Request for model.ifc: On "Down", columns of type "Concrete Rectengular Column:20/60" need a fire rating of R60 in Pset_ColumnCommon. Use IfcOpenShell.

First a look at what the model holds.

```python
import ifcopenshell
import ifcopenshell.util.element

model = ifcopenshell.open("model.ifc")
print(model.schema)
storey = next(s for s in model.by_type("IfcBuildingStorey") if s.Name == "Down")
columns = [e for e in ifcopenshell.util.element.get_decomposition(storey) if e.is_a("IfcColumn")]
seen = {}
for e in columns:
    element_type = ifcopenshell.util.element.get_type(e)
    key = (element_type.Name if element_type != e and element_type else None, ifcopenshell.util.element.get_pset(e, "Pset_ColumnCommon", "FireRating"))
    seen[key] = seen.get(key, 0) + 1
for (name, value), count in sorted(seen.items(), key=str):
    print(count, "x", name, "|", value)
```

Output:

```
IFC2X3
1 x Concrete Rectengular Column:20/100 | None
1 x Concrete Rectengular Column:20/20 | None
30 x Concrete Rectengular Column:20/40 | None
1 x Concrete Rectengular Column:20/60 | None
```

```python
import ifcopenshell
import ifcopenshell.api.pset
import ifcopenshell.util.element

model = ifcopenshell.open("model.ifc")

storey = next(s for s in model.by_type("IfcBuildingStorey") if s.Name == "Down")
columns = [e for e in ifcopenshell.util.element.get_decomposition(storey) if e.is_a("IfcColumn")]

count = 0
for e in columns:
    element_type = ifcopenshell.util.element.get_type(e)
    if element_type in (None, e) or element_type.Name != "Concrete Rectengular Column:20/60":
        continue
    # add_pset returns the element's existing set when there is one.
    pset = ifcopenshell.api.pset.add_pset(model, product=e, name="Pset_ColumnCommon")
    ifcopenshell.api.pset.edit_pset(model, pset=pset, properties={"FireRating": "R60"})
    count += 1

print(count, "columns updated")

model.write("model-out.ifc")
```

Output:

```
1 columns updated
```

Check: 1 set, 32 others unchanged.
